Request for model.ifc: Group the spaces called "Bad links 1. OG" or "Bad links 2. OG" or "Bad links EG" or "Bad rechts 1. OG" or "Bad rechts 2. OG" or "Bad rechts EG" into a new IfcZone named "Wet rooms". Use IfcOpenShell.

First a look at what the model holds.

```python
import ifcopenshell

model = ifcopenshell.open("model.ifc")
print(model.schema)
seen = {}
for space in model.by_type("IfcSpace"):
    seen[space.Name] = seen.get(space.Name, 0) + 1
for name, count in sorted(seen.items(), key=str):
    print(count, "x", name)
print("zones:", [z.Name for z in model.by_type("IfcZone")][:20])
```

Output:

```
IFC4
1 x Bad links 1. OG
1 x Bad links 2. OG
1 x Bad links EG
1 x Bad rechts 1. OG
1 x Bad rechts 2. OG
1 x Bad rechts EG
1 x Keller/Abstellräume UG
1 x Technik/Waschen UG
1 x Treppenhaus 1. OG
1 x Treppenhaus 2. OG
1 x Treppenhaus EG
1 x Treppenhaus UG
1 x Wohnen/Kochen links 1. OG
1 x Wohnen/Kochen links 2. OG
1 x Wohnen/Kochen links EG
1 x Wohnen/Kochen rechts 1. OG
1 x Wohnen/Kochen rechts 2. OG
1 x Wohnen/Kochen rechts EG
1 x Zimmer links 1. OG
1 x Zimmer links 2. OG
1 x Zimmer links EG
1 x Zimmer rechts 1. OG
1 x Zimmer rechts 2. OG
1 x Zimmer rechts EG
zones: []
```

```python
import ifcopenshell
import ifcopenshell.api.group
import ifcopenshell.api.root

model = ifcopenshell.open("model.ifc")

names = {"Bad links 1. OG", "Bad links 2. OG", "Bad links EG", "Bad rechts 1. OG", "Bad rechts 2. OG", "Bad rechts EG"}
spaces = [s for s in model.by_type("IfcSpace") if s.Name in names]

zone = ifcopenshell.api.root.create_entity(model, ifc_class="IfcZone", name="Wet rooms")
ifcopenshell.api.group.assign_group(model, products=spaces, group=zone)
print(len(spaces), "spaces in", zone.Name)

model.write("model_edited.ifc")
```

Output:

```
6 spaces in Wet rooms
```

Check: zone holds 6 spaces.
